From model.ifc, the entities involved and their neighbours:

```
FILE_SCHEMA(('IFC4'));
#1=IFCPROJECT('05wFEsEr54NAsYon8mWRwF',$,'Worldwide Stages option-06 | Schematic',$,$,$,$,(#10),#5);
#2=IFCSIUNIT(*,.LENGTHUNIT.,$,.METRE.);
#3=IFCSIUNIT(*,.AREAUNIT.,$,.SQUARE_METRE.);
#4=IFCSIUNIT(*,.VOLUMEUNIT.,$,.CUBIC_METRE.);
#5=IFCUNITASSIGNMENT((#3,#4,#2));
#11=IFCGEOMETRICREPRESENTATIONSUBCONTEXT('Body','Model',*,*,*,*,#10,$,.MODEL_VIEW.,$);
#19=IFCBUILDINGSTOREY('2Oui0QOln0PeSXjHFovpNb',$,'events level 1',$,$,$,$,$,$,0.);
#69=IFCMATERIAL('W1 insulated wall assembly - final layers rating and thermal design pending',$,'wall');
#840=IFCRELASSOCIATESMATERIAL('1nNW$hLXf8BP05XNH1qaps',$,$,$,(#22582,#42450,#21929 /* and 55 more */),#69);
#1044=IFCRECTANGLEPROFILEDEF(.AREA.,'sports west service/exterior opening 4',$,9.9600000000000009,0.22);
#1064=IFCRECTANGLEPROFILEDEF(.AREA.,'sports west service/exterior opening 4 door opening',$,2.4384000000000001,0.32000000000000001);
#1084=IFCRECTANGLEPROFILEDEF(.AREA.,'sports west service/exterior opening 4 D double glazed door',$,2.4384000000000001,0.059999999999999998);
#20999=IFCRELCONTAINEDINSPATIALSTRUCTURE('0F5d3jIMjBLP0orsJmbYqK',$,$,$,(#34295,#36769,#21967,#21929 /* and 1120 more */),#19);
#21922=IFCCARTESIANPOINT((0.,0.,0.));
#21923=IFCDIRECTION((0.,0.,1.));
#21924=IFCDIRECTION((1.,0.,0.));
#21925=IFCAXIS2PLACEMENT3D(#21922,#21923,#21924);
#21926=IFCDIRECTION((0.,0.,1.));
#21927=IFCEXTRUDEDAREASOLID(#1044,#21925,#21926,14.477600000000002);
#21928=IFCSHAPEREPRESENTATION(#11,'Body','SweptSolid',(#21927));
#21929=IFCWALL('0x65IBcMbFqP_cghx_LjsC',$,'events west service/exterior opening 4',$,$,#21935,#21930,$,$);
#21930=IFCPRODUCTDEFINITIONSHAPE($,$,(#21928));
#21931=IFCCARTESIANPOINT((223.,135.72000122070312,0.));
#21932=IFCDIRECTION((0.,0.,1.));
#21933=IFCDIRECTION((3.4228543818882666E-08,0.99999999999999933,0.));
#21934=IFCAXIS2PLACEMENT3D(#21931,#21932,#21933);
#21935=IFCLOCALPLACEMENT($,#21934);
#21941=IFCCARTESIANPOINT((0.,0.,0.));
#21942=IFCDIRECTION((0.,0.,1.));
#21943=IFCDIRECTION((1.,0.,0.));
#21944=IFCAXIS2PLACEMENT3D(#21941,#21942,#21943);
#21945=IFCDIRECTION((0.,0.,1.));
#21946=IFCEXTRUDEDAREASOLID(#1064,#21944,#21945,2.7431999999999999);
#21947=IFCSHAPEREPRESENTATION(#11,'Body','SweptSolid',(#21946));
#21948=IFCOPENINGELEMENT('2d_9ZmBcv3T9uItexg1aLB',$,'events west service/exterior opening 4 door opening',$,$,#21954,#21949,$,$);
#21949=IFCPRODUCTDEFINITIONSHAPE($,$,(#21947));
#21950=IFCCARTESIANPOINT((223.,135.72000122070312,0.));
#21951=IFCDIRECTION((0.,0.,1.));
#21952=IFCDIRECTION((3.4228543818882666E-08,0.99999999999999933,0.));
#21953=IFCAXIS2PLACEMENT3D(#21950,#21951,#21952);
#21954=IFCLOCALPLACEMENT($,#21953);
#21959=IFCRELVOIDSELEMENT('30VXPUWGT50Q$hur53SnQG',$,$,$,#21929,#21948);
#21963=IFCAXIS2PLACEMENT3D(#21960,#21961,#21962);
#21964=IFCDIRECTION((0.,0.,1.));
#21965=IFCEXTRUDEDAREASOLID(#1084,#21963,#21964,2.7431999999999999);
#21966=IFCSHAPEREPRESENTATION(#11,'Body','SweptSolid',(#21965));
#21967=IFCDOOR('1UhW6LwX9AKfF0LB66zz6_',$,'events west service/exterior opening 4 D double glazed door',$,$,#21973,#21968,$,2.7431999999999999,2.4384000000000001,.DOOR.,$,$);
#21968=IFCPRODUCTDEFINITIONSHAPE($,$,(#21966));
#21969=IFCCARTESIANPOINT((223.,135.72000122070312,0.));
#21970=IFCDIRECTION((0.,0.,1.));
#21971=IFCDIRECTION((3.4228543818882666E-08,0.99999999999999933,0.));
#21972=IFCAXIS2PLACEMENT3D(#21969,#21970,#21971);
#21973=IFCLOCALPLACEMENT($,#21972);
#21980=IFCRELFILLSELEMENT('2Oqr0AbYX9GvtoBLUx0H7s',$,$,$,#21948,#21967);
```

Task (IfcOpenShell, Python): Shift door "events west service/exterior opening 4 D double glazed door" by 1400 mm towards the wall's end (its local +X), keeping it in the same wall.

```python
import ifcopenshell
import ifcopenshell.api.geometry
import ifcopenshell.util.placement
import ifcopenshell.util.unit

model = ifcopenshell.open("model.ifc")
unit_scale = ifcopenshell.util.unit.calculate_unit_scale(model)

door = model.by_guid("1UhW6LwX9AKfF0LB66zz6_")
opening = door.FillsVoids[0].RelatingOpeningElement
wall = opening.VoidsElements[0].RelatingBuildingElement

wall_matrix = ifcopenshell.util.placement.get_local_placement(wall.ObjectPlacement)
shift = wall_matrix[:3, 0] * 1.4 / unit_scale
before = ifcopenshell.util.placement.get_local_placement(door.ObjectPlacement)[:3, 3].copy()

# The door is not placed relative to its opening, so move both.
for product in (opening, door):
    matrix = ifcopenshell.util.placement.get_local_placement(product.ObjectPlacement)
    matrix[:3, 3] += shift
    ifcopenshell.api.geometry.edit_object_placement(model, product=product, matrix=matrix, is_si=False)

after = ifcopenshell.util.placement.get_local_placement(door.ObjectPlacement)[:3, 3]
print("door moved by", (after - before).round(3) + 0.0)

model.write("model_rev.ifc")
```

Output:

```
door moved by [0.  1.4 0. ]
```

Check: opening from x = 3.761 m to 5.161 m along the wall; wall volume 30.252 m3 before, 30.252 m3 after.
